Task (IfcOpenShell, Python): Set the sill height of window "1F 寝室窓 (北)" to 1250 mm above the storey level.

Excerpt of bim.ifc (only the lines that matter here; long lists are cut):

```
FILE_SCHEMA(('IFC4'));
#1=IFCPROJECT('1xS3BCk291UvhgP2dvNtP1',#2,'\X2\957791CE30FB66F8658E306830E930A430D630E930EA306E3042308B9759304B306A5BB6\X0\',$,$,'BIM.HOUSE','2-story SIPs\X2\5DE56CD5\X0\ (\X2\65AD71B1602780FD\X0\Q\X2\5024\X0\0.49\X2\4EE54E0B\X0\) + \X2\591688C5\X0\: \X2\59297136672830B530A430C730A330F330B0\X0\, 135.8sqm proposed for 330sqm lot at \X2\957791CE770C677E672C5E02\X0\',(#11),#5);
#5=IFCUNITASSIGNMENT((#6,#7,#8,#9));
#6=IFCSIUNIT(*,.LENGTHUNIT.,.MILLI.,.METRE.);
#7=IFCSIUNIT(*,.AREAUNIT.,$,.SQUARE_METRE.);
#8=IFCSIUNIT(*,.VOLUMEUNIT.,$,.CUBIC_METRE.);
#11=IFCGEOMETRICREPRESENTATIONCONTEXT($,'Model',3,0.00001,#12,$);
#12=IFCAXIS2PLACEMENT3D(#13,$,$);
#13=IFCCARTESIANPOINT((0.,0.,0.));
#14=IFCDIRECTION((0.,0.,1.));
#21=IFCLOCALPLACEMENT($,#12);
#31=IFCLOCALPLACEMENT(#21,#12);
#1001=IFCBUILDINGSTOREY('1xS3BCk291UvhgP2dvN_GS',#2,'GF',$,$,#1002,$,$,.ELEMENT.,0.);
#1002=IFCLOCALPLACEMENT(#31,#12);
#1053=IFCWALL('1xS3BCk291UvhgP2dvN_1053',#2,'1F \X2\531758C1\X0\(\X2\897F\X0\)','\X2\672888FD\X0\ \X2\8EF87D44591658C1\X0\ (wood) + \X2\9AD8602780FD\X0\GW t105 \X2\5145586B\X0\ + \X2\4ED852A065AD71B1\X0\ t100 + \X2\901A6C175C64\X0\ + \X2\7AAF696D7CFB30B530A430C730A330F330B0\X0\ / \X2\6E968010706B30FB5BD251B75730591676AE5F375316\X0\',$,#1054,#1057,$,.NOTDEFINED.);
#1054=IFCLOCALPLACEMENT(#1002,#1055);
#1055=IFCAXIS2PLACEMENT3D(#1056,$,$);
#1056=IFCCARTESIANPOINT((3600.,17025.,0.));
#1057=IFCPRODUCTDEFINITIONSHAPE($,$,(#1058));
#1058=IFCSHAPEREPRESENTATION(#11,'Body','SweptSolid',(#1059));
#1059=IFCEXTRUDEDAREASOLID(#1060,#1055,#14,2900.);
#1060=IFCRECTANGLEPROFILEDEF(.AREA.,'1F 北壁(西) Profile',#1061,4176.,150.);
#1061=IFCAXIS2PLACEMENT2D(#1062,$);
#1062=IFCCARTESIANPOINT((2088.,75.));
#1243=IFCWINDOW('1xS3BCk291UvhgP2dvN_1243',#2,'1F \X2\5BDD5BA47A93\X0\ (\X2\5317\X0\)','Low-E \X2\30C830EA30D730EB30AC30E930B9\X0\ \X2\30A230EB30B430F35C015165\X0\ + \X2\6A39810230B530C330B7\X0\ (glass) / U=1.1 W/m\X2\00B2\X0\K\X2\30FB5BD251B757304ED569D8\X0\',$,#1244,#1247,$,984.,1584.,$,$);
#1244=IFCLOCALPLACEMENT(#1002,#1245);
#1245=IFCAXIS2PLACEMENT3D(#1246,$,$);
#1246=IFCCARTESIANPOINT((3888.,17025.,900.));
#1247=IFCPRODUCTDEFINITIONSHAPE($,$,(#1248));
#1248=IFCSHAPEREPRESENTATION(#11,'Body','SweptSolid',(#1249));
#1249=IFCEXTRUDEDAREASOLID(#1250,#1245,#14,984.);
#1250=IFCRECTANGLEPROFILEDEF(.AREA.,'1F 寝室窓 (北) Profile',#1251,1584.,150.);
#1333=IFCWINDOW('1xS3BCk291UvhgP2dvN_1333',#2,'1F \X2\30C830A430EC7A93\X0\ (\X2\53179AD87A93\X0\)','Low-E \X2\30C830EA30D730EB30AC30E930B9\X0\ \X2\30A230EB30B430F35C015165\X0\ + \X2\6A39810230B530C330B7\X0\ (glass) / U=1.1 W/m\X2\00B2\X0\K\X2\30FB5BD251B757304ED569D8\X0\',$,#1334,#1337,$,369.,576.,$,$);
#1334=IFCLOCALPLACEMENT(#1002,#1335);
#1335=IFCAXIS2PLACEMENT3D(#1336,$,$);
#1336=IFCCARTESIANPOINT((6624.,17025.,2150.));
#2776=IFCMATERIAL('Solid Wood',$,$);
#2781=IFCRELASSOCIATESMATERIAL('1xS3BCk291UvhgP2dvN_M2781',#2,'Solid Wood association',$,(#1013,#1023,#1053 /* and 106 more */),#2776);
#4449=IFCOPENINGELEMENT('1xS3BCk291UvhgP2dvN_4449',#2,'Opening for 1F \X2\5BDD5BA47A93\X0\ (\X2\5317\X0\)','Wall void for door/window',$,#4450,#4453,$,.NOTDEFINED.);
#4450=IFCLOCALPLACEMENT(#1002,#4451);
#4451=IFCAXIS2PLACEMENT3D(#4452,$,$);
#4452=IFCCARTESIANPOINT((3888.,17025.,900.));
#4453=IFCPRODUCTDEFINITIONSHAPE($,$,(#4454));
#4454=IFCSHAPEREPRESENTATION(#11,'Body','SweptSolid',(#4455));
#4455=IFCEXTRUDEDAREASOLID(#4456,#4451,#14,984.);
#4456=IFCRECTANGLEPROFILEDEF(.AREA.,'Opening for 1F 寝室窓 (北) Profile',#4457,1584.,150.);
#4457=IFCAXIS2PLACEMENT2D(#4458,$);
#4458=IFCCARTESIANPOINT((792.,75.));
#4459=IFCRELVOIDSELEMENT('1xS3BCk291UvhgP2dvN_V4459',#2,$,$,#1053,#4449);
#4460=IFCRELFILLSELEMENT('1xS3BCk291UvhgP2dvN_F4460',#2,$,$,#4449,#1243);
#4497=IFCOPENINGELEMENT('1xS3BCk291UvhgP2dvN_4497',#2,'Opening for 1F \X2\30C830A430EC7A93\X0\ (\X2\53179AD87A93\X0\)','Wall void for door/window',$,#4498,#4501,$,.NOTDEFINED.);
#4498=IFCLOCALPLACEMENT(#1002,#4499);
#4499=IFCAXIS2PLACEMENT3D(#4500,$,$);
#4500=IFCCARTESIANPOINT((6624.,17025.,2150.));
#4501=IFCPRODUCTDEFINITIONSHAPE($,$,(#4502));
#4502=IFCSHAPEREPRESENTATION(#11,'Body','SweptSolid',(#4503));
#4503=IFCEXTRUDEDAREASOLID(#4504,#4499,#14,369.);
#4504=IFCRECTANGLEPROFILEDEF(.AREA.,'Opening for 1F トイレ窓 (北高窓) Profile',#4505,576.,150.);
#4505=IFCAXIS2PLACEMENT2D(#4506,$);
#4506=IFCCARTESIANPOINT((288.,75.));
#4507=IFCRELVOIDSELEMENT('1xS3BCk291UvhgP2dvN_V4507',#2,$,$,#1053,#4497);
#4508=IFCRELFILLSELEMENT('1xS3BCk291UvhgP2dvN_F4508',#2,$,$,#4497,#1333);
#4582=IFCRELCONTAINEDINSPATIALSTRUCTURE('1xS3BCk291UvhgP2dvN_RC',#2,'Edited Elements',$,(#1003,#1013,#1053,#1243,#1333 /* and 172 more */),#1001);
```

```python
import numpy as np
import ifcopenshell
import ifcopenshell.api.geometry
import ifcopenshell.geom
import ifcopenshell.util.element
import ifcopenshell.util.placement
import ifcopenshell.util.shape
import ifcopenshell.util.unit

model = ifcopenshell.open("bim.ifc")
unit_scale = ifcopenshell.util.unit.calculate_unit_scale(model)

window = model.by_guid("1xS3BCk291UvhgP2dvN_1243")
opening = window.FillsVoids[0].RelatingOpeningElement
storey = ifcopenshell.util.element.get_container(window, ifc_class="IfcBuildingStorey")
level = ifcopenshell.util.placement.get_local_placement(storey.ObjectPlacement)[2, 3]

# The opening's origin need not be at the sill, so measure its lowest point.
shape = ifcopenshell.geom.create_shape(ifcopenshell.geom.settings(), opening)
bottom = ifcopenshell.util.shape.get_shape_bottom_elevation(shape, shape.geometry) / unit_scale
dz = level + 1.25 / unit_scale - bottom

shift = np.array([0.0, 0.0, dz])
# The window is not placed relative to its opening, so move both.
for product in (opening, window):
    matrix = ifcopenshell.util.placement.get_local_placement(product.ObjectPlacement)
    matrix[:3, 3] += shift
    ifcopenshell.api.geometry.edit_object_placement(model, product=product, matrix=matrix, is_si=False)

print(f"moved by {dz * unit_scale:+.3f} m")

model.write("bim_v2.ifc")
```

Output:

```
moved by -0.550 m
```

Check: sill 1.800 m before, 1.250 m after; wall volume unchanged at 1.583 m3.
